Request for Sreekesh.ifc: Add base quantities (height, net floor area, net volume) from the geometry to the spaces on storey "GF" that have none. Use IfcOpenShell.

First a look at what the model holds.

```python
import ifcopenshell
import ifcopenshell.util.element
import ifcopenshell.util.unit

model = ifcopenshell.open("Sreekesh.ifc")
print(model.schema)
for unit_type in ("LENGTHUNIT", "AREAUNIT", "VOLUMEUNIT"):
    print(unit_type, ifcopenshell.util.unit.calculate_unit_scale(model, unit_type))
storey = next(s for s in model.by_type("IfcBuildingStorey") if s.Name == "GF")
spaces = [e for e in ifcopenshell.util.element.get_decomposition(storey) if e.is_a("IfcSpace")]
for e in sorted(spaces, key=lambda e: e.id()):
    print(e.id(), e.is_a(), e.Name, list(ifcopenshell.util.element.get_psets(e, qtos_only=True)), sep=" | ")
```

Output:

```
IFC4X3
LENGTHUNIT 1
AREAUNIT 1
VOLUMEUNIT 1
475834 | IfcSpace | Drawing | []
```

```python
import ifcopenshell
import ifcopenshell.api.pset
import ifcopenshell.geom
import ifcopenshell.util.element
import ifcopenshell.util.shape
import ifcopenshell.util.unit

model = ifcopenshell.open("Sreekesh.ifc")
unit_scale = ifcopenshell.util.unit.calculate_unit_scale(model)
area_scale = ifcopenshell.util.unit.calculate_unit_scale(model, "AREAUNIT")
volume_scale = ifcopenshell.util.unit.calculate_unit_scale(model, "VOLUMEUNIT")
settings = ifcopenshell.geom.settings()

storey = next(s for s in model.by_type("IfcBuildingStorey") if s.Name == "GF")
spaces = [e for e in ifcopenshell.util.element.get_decomposition(storey) if e.is_a("IfcSpace")]

for e in sorted(spaces, key=lambda e: e.id()):
    if ifcopenshell.util.element.get_psets(e, qtos_only=True, should_inherit=False):
        continue
    # Geometry comes back in metres, in the element's own axes.
    shape = ifcopenshell.geom.create_shape(settings, e)
    values = {
        "Height": ifcopenshell.util.shape.get_z(shape.geometry) / unit_scale,
        "NetFloorArea": ifcopenshell.util.shape.get_footprint_area(shape.geometry) / area_scale,
        "NetVolume": ifcopenshell.util.shape.get_volume(shape.geometry) / volume_scale,
    }
    qto = ifcopenshell.api.pset.add_qto(model, product=e, name="Qto_SpaceBaseQuantities")
    ifcopenshell.api.pset.edit_qto(model, qto=qto, properties=values)
    print(e.id(), {k: round(v, 3) for k, v in values.items()})

model.write("Sreekesh-out.ifc")
```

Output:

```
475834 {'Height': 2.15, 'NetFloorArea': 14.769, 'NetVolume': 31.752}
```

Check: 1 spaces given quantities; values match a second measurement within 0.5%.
